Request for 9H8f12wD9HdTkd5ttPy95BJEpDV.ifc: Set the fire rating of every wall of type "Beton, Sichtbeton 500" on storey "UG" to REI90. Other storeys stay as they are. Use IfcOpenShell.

First a look at what the model holds.

```python
import ifcopenshell
import ifcopenshell.util.element

model = ifcopenshell.open("9H8f12wD9HdTkd5ttPy95BJEpDV.ifc")
print(model.schema)
storey = next(s for s in model.by_type("IfcBuildingStorey") if s.Name == "UG")
walls = [e for e in ifcopenshell.util.element.get_decomposition(storey) if e.is_a("IfcWall")]
seen = {}
for e in walls:
    element_type = ifcopenshell.util.element.get_type(e)
    key = (element_type.Name if element_type != e and element_type else None, ifcopenshell.util.element.get_pset(e, "Pset_WallCommon", "FireRating"))
    seen[key] = seen.get(key, 0) + 1
for (name, value), count in sorted(seen.items(), key=str):
    print(count, "x", name, "|", value)
```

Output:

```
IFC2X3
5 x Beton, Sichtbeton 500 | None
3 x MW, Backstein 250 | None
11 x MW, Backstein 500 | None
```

```python
import ifcopenshell
import ifcopenshell.api.pset
import ifcopenshell.util.element

model = ifcopenshell.open("9H8f12wD9HdTkd5ttPy95BJEpDV.ifc")

storey = next(s for s in model.by_type("IfcBuildingStorey") if s.Name == "UG")
walls = [e for e in ifcopenshell.util.element.get_decomposition(storey) if e.is_a("IfcWall")]

count = 0
for e in walls:
    element_type = ifcopenshell.util.element.get_type(e)
    if element_type in (None, e) or element_type.Name != "Beton, Sichtbeton 500":
        continue
    # add_pset returns the element's existing set when there is one.
    pset = ifcopenshell.api.pset.add_pset(model, product=e, name="Pset_WallCommon")
    ifcopenshell.api.pset.edit_pset(model, pset=pset, properties={"FireRating": "REI90"})
    count += 1

print(count, "walls updated")

model.write("9H8f12wD9HdTkd5ttPy95BJEpDV-out.ifc")
```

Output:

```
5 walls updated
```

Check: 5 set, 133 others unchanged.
